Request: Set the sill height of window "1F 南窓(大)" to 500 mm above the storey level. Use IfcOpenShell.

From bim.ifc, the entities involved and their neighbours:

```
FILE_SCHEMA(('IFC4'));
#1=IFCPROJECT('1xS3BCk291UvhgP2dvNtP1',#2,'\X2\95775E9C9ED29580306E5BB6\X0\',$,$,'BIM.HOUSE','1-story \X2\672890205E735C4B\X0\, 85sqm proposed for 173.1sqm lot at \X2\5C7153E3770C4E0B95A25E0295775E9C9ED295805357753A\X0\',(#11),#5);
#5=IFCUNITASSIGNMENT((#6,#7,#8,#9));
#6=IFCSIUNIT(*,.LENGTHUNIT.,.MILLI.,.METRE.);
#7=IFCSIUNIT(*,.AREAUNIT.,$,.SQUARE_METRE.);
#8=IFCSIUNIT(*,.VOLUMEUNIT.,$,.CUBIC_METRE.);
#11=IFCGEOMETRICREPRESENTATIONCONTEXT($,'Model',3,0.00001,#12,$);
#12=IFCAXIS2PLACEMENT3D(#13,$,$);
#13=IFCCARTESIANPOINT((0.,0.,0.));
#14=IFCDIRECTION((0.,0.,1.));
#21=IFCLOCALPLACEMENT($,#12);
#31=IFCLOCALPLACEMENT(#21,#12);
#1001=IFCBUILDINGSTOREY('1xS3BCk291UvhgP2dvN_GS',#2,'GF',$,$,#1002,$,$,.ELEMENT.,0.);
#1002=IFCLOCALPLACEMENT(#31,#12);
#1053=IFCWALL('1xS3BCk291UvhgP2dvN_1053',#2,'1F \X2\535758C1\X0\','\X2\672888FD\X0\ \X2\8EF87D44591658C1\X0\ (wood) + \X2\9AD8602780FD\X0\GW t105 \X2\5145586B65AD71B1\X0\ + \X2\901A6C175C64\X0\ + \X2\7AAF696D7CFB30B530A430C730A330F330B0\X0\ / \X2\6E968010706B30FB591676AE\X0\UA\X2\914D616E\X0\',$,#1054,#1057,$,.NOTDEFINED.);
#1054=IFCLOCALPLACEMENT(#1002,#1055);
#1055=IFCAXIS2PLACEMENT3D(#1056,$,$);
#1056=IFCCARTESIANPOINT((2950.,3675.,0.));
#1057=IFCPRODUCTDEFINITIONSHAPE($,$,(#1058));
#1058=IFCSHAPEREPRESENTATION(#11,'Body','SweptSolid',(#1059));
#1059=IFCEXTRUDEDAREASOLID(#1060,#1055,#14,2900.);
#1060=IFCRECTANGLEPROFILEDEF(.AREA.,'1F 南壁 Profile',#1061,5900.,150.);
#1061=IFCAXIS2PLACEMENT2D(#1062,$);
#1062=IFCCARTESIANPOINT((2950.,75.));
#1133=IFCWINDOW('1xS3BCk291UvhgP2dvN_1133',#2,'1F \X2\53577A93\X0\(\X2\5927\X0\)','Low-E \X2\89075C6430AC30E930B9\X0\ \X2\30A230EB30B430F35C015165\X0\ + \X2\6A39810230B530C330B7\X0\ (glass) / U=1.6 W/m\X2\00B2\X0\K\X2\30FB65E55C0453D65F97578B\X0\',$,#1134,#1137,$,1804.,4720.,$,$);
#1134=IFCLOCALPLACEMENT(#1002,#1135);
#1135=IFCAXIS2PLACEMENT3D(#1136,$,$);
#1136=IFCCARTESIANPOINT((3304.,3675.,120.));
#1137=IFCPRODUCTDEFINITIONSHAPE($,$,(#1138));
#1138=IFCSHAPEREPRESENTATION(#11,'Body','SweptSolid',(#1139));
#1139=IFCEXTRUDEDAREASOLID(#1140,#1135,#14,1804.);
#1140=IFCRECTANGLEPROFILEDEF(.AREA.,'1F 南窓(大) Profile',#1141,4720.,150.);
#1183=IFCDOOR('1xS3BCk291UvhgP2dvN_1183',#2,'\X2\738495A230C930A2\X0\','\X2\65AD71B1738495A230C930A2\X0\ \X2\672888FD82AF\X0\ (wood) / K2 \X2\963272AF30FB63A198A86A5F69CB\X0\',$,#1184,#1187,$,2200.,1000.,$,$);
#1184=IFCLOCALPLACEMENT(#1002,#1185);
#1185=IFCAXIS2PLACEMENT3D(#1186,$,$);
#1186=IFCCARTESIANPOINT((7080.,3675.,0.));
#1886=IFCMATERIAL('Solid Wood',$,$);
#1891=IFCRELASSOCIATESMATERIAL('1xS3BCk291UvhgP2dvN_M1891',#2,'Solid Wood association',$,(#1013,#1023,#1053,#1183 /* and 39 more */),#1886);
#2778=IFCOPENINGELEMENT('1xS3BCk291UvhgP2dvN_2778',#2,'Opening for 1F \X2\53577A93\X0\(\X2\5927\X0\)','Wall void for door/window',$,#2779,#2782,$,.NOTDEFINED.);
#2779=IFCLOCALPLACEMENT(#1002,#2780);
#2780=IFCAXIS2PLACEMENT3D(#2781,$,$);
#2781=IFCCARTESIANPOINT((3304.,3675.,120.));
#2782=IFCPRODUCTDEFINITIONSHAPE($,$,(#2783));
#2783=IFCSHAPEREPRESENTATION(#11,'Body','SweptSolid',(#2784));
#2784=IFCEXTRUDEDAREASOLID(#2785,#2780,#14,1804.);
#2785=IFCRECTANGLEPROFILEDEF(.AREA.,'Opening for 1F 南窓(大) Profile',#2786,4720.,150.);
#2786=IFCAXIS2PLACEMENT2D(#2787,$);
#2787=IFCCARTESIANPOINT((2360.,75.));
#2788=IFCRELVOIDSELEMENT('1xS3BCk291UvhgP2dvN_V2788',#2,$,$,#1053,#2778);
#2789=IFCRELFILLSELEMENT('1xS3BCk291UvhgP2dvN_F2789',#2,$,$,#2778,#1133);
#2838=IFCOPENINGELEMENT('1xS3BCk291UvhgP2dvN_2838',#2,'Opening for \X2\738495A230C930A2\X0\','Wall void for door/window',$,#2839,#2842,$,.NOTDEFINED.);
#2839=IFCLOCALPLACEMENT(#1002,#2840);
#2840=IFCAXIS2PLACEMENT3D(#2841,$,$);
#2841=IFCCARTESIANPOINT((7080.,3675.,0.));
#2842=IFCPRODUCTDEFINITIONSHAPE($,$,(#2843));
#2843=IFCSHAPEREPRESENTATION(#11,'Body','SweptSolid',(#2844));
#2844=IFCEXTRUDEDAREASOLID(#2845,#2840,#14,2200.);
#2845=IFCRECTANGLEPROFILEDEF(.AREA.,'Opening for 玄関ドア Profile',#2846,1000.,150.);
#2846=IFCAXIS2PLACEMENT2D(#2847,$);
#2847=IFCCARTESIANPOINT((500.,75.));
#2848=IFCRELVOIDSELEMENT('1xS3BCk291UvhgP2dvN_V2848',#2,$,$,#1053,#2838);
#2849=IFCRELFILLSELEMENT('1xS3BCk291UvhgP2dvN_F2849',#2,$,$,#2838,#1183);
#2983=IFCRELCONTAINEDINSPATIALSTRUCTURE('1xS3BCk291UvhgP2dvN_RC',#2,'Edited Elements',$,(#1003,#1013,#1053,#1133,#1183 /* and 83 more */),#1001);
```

```python
import numpy as np
import ifcopenshell
import ifcopenshell.api.geometry
import ifcopenshell.geom
import ifcopenshell.util.element
import ifcopenshell.util.placement
import ifcopenshell.util.shape
import ifcopenshell.util.unit

model = ifcopenshell.open("bim.ifc")
unit_scale = ifcopenshell.util.unit.calculate_unit_scale(model)

window = model.by_guid("1xS3BCk291UvhgP2dvN_1133")
opening = window.FillsVoids[0].RelatingOpeningElement
storey = ifcopenshell.util.element.get_container(window, ifc_class="IfcBuildingStorey")
level = ifcopenshell.util.placement.get_local_placement(storey.ObjectPlacement)[2, 3]

# The opening's origin need not be at the sill, so measure its lowest point.
shape = ifcopenshell.geom.create_shape(ifcopenshell.geom.settings(), opening)
bottom = ifcopenshell.util.shape.get_shape_bottom_elevation(shape, shape.geometry) / unit_scale
dz = level + 0.5 / unit_scale - bottom

shift = np.array([0.0, 0.0, dz])
# The window is not placed relative to its opening, so move both.
for product in (opening, window):
    matrix = ifcopenshell.util.placement.get_local_placement(product.ObjectPlacement)
    matrix[:3, 3] += shift
    ifcopenshell.api.geometry.edit_object_placement(model, product=product, matrix=matrix, is_si=False)

print(f"moved by {dz * unit_scale:+.3f} m")

model.write("bim-out.ifc")
```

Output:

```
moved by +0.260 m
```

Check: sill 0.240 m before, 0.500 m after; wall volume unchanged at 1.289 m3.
